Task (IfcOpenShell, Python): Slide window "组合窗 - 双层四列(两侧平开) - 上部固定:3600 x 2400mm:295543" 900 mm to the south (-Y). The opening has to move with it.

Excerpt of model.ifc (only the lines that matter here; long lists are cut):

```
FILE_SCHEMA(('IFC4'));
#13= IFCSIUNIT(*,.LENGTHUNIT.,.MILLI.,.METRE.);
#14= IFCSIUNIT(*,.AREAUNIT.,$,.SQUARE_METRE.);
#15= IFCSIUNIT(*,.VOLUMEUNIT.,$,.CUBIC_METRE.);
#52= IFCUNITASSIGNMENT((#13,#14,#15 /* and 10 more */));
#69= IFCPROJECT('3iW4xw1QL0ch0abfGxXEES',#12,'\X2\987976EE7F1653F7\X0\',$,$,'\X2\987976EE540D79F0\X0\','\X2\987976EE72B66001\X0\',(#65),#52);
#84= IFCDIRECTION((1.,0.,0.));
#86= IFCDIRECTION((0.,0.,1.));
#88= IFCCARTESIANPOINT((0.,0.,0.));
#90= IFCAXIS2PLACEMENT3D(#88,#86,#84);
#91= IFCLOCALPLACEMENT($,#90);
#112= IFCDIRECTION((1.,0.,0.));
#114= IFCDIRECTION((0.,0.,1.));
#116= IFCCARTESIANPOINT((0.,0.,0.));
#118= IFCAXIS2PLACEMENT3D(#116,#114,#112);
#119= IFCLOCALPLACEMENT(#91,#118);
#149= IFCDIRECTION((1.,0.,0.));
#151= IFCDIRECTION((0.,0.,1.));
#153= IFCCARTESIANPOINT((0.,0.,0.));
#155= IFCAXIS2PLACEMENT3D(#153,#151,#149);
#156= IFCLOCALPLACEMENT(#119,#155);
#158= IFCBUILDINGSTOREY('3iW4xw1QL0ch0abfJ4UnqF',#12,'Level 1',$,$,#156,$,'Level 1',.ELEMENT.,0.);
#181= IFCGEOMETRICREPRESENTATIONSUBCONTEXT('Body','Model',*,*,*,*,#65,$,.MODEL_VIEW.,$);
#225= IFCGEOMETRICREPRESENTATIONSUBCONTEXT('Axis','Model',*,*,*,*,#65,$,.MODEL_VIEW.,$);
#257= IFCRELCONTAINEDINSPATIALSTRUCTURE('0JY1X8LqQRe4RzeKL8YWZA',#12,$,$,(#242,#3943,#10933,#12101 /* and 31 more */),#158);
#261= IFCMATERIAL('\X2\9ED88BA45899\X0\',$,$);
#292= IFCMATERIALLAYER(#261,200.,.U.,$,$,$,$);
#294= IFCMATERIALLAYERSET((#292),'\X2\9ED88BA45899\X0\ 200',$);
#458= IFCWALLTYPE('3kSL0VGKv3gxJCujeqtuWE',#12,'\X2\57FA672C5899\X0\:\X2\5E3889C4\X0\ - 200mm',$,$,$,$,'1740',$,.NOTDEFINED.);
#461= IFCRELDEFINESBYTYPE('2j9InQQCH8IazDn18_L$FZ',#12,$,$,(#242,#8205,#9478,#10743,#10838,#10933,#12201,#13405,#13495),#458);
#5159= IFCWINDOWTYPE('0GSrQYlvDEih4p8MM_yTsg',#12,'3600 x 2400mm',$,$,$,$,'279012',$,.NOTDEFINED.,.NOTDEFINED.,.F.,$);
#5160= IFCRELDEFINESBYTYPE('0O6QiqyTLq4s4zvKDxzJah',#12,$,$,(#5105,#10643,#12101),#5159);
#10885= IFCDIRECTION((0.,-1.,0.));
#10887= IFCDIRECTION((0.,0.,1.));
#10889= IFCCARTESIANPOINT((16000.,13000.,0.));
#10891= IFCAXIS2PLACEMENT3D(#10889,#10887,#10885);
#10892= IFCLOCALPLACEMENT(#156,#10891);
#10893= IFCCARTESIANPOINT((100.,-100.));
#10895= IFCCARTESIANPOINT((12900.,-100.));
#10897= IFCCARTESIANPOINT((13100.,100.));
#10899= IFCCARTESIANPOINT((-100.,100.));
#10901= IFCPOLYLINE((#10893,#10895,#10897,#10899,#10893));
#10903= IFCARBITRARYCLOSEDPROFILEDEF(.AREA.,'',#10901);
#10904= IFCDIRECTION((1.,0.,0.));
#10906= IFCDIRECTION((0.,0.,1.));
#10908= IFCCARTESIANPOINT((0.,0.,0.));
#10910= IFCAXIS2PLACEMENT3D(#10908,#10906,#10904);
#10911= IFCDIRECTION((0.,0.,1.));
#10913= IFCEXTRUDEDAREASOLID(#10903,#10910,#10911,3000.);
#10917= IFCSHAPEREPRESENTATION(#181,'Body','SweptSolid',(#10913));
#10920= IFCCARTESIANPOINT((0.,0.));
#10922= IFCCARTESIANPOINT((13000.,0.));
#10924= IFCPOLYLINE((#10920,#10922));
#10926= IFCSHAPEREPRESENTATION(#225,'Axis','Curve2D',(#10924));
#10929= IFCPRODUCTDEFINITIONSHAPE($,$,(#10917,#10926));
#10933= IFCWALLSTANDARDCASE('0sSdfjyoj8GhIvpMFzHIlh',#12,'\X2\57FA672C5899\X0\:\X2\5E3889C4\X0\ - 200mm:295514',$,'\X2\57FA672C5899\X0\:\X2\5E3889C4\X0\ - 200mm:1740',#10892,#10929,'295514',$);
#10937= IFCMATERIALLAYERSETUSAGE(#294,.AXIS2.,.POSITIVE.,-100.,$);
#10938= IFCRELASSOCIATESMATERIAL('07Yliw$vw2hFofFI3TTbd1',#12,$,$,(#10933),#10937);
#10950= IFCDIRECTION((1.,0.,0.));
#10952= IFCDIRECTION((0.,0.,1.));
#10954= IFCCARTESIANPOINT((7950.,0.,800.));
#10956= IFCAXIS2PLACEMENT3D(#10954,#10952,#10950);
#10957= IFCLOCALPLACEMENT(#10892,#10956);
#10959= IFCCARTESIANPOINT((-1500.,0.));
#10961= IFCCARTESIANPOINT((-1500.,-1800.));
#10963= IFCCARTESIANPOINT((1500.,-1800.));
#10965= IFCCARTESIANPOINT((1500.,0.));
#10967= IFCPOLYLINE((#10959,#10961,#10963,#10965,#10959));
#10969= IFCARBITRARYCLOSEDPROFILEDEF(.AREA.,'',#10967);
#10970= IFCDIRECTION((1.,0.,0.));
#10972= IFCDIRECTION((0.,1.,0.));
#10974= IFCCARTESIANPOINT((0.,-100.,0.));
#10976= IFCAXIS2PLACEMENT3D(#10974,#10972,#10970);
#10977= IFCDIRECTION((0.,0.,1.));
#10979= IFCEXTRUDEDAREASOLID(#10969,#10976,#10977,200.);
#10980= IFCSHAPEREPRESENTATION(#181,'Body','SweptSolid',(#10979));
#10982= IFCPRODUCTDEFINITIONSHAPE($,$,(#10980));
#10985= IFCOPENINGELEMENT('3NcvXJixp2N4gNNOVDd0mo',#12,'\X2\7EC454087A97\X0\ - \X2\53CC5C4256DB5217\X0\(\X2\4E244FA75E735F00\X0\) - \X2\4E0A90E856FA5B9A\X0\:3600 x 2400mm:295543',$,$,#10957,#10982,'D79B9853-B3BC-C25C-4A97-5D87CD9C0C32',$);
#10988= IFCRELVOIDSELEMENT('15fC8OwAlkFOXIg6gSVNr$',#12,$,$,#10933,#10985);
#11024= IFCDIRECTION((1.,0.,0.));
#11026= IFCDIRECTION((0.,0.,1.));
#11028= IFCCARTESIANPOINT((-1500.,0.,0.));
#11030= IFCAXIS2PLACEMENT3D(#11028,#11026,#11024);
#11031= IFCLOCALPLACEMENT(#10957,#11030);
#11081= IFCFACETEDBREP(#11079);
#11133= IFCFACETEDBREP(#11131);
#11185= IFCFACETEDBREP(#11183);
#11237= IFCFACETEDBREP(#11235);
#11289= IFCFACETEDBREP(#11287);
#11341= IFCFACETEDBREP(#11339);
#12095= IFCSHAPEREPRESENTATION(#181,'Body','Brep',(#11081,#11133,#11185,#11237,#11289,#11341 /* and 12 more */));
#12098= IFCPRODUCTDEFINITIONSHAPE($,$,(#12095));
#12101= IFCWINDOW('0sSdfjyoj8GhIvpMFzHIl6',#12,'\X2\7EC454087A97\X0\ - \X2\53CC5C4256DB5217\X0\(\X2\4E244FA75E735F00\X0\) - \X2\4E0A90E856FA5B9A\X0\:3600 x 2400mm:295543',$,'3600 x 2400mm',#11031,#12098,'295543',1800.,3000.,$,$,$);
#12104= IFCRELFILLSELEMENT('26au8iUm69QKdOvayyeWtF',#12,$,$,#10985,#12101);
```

```python
import ifcopenshell
import ifcopenshell.api.geometry
import ifcopenshell.util.placement
import ifcopenshell.util.unit

model = ifcopenshell.open("model.ifc")
unit_scale = ifcopenshell.util.unit.calculate_unit_scale(model)

window = model.by_guid("0sSdfjyoj8GhIvpMFzHIl6")
opening = window.FillsVoids[0].RelatingOpeningElement
wall = opening.VoidsElements[0].RelatingBuildingElement

wall_matrix = ifcopenshell.util.placement.get_local_placement(wall.ObjectPlacement)
shift = wall_matrix[:3, 0] * 0.9 / unit_scale
before = ifcopenshell.util.placement.get_local_placement(window.ObjectPlacement)[:3, 3].copy()

# The window is placed relative to its opening, so it follows when the opening moves.
matrix = ifcopenshell.util.placement.get_local_placement(opening.ObjectPlacement)
matrix[:3, 3] += shift
ifcopenshell.api.geometry.edit_object_placement(
    model, product=opening, matrix=matrix, is_si=False, should_transform_children=True
)

after = ifcopenshell.util.placement.get_local_placement(window.ObjectPlacement)[:3, 3]
print("window moved by", (after - before).round(3) + 0.0)

model.write("model-out.ifc")
```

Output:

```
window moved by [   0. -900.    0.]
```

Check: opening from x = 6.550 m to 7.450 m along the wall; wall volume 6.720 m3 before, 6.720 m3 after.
